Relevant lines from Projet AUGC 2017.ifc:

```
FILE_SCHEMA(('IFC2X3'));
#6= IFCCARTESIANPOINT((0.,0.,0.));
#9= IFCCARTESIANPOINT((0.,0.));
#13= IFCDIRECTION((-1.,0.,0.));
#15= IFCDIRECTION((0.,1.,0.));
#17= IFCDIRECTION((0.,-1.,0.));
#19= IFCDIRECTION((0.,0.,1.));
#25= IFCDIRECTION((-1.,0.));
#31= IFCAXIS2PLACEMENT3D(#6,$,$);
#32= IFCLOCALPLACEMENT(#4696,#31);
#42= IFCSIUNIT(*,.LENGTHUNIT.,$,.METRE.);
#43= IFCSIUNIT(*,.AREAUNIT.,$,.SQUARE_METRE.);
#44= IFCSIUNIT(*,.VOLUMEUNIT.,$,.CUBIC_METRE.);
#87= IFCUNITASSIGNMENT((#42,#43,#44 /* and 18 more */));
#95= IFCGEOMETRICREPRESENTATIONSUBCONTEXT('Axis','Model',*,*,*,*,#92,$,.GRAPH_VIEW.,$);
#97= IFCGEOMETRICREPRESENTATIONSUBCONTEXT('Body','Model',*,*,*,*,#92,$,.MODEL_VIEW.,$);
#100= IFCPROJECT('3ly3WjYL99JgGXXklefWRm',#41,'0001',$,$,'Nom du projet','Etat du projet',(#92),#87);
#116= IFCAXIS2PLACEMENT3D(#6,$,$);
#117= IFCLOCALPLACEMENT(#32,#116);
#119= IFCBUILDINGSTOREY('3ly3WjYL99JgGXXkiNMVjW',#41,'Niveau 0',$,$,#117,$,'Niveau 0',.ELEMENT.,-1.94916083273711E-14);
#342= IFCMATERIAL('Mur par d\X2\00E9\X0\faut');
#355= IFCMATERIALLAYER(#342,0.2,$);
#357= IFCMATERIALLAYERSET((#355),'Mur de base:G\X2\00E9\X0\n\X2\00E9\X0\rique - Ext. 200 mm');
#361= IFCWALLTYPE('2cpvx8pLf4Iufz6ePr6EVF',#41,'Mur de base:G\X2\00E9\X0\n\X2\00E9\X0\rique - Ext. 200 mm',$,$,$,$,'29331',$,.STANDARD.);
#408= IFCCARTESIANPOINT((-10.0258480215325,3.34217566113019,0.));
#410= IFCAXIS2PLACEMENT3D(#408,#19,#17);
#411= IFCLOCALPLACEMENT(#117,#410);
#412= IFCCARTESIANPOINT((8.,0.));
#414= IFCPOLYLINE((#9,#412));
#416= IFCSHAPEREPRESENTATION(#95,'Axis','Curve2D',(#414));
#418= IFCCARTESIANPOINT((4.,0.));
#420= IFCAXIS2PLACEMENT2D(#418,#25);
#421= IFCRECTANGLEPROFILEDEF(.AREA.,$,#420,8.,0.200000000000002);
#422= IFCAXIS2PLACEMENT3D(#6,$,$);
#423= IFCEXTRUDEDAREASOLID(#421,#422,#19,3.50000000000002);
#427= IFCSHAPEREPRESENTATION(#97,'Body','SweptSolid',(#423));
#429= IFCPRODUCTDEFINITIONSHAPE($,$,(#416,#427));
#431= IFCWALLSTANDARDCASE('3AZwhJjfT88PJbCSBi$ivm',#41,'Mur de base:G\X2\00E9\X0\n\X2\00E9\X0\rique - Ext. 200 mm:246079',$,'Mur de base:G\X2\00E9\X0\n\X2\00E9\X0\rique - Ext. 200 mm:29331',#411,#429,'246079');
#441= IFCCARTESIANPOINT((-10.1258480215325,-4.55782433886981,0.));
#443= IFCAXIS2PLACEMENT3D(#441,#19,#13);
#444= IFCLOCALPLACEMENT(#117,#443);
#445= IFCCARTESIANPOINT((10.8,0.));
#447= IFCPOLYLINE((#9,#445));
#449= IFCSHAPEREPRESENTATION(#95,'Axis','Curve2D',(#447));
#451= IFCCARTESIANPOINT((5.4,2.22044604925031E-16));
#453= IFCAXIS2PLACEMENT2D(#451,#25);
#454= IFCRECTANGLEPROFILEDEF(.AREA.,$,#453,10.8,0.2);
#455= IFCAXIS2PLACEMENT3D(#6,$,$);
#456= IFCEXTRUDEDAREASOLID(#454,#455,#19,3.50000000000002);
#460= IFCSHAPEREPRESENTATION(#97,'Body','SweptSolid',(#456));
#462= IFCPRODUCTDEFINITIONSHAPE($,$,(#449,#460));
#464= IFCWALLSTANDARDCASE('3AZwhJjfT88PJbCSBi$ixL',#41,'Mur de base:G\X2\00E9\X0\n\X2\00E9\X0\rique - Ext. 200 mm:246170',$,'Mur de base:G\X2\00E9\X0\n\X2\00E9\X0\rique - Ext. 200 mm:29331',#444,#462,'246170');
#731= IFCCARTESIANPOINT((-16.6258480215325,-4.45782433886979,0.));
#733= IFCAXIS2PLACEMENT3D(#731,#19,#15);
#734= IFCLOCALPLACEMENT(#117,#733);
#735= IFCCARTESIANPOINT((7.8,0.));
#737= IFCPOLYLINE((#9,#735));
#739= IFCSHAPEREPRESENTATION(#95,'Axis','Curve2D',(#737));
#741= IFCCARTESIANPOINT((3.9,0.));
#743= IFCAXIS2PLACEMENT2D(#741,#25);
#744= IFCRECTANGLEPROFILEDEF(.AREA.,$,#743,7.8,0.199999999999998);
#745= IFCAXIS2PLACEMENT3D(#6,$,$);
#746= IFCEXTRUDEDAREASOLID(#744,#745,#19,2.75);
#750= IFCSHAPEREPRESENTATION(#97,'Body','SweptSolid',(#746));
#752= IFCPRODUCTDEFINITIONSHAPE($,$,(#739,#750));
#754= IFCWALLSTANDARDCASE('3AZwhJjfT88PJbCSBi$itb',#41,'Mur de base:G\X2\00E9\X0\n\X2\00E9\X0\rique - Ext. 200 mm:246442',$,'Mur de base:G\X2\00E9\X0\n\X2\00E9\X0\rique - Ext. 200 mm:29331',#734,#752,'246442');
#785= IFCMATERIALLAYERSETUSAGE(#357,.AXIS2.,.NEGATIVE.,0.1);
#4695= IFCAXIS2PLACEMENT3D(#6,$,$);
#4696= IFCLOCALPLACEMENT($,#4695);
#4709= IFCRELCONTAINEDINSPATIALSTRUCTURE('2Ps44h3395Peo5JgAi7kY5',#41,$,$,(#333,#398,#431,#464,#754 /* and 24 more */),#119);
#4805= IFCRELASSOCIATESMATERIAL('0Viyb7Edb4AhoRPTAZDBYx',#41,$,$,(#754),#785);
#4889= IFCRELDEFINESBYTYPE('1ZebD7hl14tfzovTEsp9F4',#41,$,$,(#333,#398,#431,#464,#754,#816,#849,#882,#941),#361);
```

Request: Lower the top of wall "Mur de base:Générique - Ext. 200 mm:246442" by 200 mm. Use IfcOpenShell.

```python
import ifcopenshell
import ifcopenshell.geom
import ifcopenshell.util.representation
import ifcopenshell.util.shape

model = ifcopenshell.open("Projet AUGC 2017.ifc")
settings = ifcopenshell.geom.settings()


def volume(element):
    """Net volume in cubic metres, openings subtracted."""
    shape = ifcopenshell.geom.create_shape(settings, element)
    return ifcopenshell.util.shape.get_volume(shape.geometry)


wall = model.by_guid("3AZwhJjfT88PJbCSBi$itb")
before = volume(wall)

body = ifcopenshell.util.representation.get_representation(wall, "Model", "Body")
solid = body.Items[0]
old_height = solid.Depth
solid.Depth -= 0.2
after = volume(wall)

print(f"height {old_height:g} -> {solid.Depth:g}, volume {before:.3f} -> {after:.3f} m3")

model.write("Projet AUGC 2017_rev.ifc")
```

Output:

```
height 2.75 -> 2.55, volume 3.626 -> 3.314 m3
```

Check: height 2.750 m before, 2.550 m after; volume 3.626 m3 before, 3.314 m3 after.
